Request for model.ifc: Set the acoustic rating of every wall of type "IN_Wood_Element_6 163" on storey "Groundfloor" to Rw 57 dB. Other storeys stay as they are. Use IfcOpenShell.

First a look at what the model holds.

```python
import ifcopenshell
import ifcopenshell.util.element

model = ifcopenshell.open("model.ifc")
print(model.schema)
storey = next(s for s in model.by_type("IfcBuildingStorey") if s.Name == "Groundfloor")
walls = [e for e in ifcopenshell.util.element.get_decomposition(storey) if e.is_a("IfcWall")]
seen = {}
for e in walls:
    element_type = ifcopenshell.util.element.get_type(e)
    key = (element_type.Name if element_type != e and element_type else None, ifcopenshell.util.element.get_pset(e, "Pset_WallCommon", "AcousticRating"))
    seen[key] = seen.get(key, 0) + 1
for (name, value), count in sorted(seen.items(), key=str):
    print(count, "x", name, "|", value)
```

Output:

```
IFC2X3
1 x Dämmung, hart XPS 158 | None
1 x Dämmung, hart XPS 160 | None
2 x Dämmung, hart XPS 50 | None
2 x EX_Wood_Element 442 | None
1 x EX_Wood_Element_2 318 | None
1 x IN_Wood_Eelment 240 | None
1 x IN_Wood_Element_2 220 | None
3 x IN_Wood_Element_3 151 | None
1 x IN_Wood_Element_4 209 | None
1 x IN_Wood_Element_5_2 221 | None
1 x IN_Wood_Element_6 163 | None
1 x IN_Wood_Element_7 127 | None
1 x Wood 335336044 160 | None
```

```python
import ifcopenshell
import ifcopenshell.api.pset
import ifcopenshell.util.element

model = ifcopenshell.open("model.ifc")

storey = next(s for s in model.by_type("IfcBuildingStorey") if s.Name == "Groundfloor")
walls = [e for e in ifcopenshell.util.element.get_decomposition(storey) if e.is_a("IfcWall")]

count = 0
for e in walls:
    element_type = ifcopenshell.util.element.get_type(e)
    if element_type in (None, e) or element_type.Name != "IN_Wood_Element_6 163":
        continue
    # add_pset returns the element's existing set when there is one.
    pset = ifcopenshell.api.pset.add_pset(model, product=e, name="Pset_WallCommon")
    ifcopenshell.api.pset.edit_pset(model, pset=pset, properties={"AcousticRating": "Rw 57 dB"})
    count += 1

print(count, "walls updated")

model.write("model_edited.ifc")
```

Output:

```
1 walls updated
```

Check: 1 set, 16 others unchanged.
